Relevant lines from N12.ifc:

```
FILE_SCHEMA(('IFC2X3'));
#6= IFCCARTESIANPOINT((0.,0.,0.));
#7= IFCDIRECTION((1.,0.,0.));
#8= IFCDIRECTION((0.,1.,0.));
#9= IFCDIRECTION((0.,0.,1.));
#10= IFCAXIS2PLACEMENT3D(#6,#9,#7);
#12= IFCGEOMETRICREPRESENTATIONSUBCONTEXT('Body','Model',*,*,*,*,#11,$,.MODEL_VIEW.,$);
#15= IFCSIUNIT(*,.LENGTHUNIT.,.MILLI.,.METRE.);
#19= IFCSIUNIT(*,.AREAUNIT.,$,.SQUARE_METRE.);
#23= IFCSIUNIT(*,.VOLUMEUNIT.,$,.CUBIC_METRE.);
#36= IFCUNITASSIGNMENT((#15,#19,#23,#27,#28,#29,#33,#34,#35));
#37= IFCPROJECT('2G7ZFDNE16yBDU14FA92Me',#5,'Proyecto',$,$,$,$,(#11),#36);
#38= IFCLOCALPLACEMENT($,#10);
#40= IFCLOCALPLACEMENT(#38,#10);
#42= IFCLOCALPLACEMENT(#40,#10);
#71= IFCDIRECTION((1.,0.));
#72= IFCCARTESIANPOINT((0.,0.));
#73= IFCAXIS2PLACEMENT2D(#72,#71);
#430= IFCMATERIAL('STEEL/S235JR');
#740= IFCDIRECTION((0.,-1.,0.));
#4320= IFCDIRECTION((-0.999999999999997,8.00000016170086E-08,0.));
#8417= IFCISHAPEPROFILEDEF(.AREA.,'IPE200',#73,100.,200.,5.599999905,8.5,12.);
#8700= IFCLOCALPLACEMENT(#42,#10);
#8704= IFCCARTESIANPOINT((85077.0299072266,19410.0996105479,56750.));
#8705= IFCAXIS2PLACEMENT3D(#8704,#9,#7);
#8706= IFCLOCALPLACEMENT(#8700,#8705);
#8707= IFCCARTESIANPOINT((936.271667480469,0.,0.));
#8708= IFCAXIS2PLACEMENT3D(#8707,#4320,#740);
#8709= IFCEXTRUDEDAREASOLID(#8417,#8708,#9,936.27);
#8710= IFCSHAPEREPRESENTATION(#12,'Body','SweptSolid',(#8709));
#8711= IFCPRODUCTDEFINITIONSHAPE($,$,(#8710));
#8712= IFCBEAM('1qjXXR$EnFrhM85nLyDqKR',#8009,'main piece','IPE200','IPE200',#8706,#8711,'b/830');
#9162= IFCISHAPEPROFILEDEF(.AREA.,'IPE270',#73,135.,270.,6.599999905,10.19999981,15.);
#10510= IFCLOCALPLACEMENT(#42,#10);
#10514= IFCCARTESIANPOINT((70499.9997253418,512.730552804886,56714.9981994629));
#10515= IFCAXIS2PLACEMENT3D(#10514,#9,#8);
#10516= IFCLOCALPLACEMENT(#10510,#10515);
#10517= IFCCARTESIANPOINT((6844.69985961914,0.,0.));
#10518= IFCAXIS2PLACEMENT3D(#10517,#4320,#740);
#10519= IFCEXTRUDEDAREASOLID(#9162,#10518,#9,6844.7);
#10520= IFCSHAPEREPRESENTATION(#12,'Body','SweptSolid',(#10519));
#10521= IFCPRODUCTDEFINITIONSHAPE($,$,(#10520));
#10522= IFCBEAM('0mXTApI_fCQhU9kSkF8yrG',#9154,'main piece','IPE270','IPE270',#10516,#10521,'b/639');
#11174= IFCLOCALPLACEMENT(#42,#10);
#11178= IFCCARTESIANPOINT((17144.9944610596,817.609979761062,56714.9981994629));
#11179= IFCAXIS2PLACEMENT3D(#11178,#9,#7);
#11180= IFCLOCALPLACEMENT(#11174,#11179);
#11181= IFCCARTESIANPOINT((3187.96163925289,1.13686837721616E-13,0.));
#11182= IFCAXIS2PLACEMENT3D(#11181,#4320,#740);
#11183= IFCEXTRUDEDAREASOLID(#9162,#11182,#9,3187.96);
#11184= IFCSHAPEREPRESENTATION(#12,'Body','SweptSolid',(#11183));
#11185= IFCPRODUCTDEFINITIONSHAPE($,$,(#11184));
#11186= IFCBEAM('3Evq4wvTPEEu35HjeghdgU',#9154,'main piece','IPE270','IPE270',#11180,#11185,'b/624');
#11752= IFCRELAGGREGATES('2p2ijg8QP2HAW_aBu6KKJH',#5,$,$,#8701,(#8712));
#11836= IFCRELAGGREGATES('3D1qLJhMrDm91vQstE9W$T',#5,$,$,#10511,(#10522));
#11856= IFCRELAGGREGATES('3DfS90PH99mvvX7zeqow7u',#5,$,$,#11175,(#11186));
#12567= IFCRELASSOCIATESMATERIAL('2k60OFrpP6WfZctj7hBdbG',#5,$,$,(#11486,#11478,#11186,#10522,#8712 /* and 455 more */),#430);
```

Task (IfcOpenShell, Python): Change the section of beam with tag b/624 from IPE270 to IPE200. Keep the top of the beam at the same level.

```python
import ifcopenshell
import ifcopenshell.util.element
import ifcopenshell.util.representation

model = ifcopenshell.open("N12.ifc")

member = model.by_guid("3Evq4wvTPEEu35HjeghdgU")
source = next(p for p in model.by_type("IfcIShapeProfileDef") if p.ProfileName == "IPE200")

body = ifcopenshell.util.representation.get_representation(member, "Model", "Body")
solid = body.Items[0]
old_profile = solid.SweptArea

# Copy the section's sizes but keep this member's own profile position.
profile = ifcopenshell.util.element.copy(model, source)
# Profiles are centred, so shift by half the change in depth to hold the top.
shift = (old_profile.OverallDepth - profile.OverallDepth) / 2
x, y = old_profile.Position.Location.Coordinates
up = (0.0, 1.0)  # upwards, in the solid's own plane
location = model.createIfcCartesianPoint((x + up[0] * shift, y + up[1] * shift))
profile.Position = model.createIfcAxis2Placement2D(location, old_profile.Position.RefDirection)
solid.SweptArea = profile
if not model.get_total_inverses(old_profile):
    ifcopenshell.util.element.remove_deep2(model, old_profile)
member.Description = member.Description.replace("IPE270", "IPE200")
member.ObjectType = member.ObjectType.replace("IPE270", "IPE200")

print(solid.SweptArea)

model.write("N12_edited.ifc")
```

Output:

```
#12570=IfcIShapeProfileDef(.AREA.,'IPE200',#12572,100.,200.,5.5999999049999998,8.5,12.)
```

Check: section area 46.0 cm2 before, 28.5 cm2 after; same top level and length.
